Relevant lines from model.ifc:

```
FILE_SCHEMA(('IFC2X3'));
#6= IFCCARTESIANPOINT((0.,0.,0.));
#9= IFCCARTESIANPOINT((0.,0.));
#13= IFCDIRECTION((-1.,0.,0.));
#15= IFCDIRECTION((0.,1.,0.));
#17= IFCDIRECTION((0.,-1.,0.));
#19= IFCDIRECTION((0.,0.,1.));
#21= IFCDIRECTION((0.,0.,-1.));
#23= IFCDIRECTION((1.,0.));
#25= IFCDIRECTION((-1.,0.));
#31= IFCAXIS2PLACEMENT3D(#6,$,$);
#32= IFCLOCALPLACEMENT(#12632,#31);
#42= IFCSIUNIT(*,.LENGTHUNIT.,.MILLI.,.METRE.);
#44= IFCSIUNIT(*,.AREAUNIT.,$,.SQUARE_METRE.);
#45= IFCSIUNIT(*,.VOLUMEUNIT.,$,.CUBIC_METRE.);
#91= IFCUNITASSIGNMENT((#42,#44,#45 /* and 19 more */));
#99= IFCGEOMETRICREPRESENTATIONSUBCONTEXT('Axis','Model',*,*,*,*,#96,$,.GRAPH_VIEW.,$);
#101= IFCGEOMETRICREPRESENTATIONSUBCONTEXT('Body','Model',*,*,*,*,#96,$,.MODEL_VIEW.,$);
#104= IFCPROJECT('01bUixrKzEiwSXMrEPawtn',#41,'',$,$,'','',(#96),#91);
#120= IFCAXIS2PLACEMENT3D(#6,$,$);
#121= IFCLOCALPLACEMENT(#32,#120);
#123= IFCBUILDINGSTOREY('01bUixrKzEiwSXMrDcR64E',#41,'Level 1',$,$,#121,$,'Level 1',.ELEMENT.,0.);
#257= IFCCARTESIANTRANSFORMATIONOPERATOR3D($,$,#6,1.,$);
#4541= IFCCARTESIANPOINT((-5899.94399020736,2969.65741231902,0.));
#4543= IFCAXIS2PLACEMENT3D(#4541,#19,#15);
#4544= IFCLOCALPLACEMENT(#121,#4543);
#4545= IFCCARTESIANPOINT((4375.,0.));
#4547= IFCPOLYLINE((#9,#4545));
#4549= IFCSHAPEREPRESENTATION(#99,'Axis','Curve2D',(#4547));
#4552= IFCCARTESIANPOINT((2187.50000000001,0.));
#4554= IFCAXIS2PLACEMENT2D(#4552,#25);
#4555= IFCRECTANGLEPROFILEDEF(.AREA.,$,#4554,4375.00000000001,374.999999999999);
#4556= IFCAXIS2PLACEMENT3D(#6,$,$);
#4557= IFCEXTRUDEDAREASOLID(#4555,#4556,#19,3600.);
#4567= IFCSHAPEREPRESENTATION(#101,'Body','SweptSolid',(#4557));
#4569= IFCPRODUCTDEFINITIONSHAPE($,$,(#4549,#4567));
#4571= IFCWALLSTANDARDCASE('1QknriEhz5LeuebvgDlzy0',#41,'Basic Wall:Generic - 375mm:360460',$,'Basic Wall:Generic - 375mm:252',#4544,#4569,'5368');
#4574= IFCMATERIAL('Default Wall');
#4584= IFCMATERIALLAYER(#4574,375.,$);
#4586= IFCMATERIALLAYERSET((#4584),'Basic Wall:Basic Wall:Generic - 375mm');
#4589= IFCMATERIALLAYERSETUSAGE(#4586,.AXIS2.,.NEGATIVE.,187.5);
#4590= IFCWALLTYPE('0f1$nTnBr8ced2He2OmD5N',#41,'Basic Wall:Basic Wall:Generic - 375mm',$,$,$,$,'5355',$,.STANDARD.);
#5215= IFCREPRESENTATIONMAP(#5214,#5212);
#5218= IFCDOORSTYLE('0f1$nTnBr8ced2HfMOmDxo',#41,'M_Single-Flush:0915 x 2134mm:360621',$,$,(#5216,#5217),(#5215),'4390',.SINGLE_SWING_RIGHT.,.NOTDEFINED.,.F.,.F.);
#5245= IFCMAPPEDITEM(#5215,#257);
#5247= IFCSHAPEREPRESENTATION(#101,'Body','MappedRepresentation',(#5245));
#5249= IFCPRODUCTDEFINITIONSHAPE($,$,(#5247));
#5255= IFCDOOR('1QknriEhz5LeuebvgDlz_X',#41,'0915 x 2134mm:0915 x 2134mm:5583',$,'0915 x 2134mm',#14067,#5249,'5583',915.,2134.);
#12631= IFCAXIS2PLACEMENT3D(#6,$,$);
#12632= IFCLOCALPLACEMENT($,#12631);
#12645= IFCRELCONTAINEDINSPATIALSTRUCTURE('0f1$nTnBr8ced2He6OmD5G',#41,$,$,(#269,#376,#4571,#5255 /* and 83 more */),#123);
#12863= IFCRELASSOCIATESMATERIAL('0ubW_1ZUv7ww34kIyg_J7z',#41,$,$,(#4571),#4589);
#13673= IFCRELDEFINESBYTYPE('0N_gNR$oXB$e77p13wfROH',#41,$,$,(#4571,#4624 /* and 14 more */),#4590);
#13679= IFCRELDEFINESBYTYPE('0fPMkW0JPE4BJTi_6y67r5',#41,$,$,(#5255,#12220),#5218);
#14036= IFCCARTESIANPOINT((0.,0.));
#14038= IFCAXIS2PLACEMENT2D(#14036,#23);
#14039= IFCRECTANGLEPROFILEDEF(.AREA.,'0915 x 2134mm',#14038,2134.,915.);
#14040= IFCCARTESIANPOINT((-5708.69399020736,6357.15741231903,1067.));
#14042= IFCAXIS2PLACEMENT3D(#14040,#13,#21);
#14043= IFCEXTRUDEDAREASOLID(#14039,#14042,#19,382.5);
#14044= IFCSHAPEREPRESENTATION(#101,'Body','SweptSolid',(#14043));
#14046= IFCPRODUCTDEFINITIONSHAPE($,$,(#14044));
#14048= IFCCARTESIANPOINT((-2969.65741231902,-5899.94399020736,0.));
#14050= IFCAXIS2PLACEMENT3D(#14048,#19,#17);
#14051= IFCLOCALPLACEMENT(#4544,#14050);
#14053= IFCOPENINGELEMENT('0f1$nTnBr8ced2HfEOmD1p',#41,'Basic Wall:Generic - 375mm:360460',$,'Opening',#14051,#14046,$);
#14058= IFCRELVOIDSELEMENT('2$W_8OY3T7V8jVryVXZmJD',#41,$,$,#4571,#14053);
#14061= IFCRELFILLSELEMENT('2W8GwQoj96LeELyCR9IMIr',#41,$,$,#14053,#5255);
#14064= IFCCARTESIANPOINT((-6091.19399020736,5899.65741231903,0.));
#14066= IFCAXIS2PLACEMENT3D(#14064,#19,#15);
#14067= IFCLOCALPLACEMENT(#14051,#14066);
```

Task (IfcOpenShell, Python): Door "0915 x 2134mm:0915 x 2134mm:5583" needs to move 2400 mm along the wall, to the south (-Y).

```python
import ifcopenshell
import ifcopenshell.api.geometry
import ifcopenshell.util.placement

model = ifcopenshell.open("model.ifc")

door = model.by_id(5255)
opening = door.FillsVoids[0].RelatingOpeningElement
wall = opening.VoidsElements[0].RelatingBuildingElement

wall_matrix = ifcopenshell.util.placement.get_local_placement(wall.ObjectPlacement)
shift = wall_matrix[:3, 0] * -2400.0
before = ifcopenshell.util.placement.get_local_placement(door.ObjectPlacement)[:3, 3].copy()

# The door is placed relative to its opening, so it follows when the opening moves.
matrix = ifcopenshell.util.placement.get_local_placement(opening.ObjectPlacement)
matrix[:3, 3] += shift
ifcopenshell.api.geometry.edit_object_placement(
    model, product=opening, matrix=matrix, is_si=False, should_transform_children=True
)

after = ifcopenshell.util.placement.get_local_placement(door.ObjectPlacement)[:3, 3]
print("door moved by", (after - before).round(3) + 0.0)

model.write("model_rev.ifc")
```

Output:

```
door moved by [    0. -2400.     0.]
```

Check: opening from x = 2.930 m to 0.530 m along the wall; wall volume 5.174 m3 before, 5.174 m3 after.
